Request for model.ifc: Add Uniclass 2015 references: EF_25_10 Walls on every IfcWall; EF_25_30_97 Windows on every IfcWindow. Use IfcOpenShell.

First a look at what the model holds.

```python
import ifcopenshell

model = ifcopenshell.open("model.ifc")
print(model.schema)
print("classifications:", [c.Name for c in model.by_type("IfcClassification")])
for ifc_class in ("IfcDoor", "IfcRoof", "IfcStair", "IfcWall", "IfcWindow"):
    print(ifc_class, len(model.by_type(ifc_class)))
```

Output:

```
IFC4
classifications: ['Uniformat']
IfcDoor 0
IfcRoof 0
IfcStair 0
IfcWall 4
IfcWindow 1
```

```python
import ifcopenshell
import ifcopenshell.api.classification

model = ifcopenshell.open("model.ifc")

system = ifcopenshell.api.classification.add_classification(model, classification="Uniclass 2015")

codes = {
    "IfcWall": ("EF_25_10", "Walls"),
    "IfcWindow": ("EF_25_30_97", "Windows"),
}
for ifc_class, (code, name) in codes.items():
    products = model.by_type(ifc_class)
    ifcopenshell.api.classification.add_reference(
        model, products=products, classification=system, identification=code, name=name
    )
    print(code, len(products))

model.write("model_rev.ifc")
```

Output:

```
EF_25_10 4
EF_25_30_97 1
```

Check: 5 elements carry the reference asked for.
